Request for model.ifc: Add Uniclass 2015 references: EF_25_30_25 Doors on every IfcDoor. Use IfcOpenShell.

First a look at what the model holds.

```python
import ifcopenshell

model = ifcopenshell.open("model.ifc")
print(model.schema)
print("classifications:", [c.Name for c in model.by_type("IfcClassification")])
for ifc_class in ("IfcDoor", "IfcRoof", "IfcStair", "IfcWall", "IfcWindow"):
    print(ifc_class, len(model.by_type(ifc_class)))
```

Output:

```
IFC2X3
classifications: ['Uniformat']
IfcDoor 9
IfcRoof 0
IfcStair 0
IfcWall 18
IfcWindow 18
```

```python
import ifcopenshell
import ifcopenshell.api.classification

model = ifcopenshell.open("model.ifc")

# IFC2X3 requires Source and Edition and has no link from the project to the system.
system = model.create_entity("IfcClassification", Source="NBS", Edition="2015", Name="Uniclass 2015")

codes = {
    "IfcDoor": ("EF_25_30_25", "Doors"),
}
for ifc_class, (code, name) in codes.items():
    products = model.by_type(ifc_class)
    ifcopenshell.api.classification.add_reference(
        model, products=products, classification=system, identification=code, name=name
    )
    print(code, len(products))

model.write("model_v2.ifc")
```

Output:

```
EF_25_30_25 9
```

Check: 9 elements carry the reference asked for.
